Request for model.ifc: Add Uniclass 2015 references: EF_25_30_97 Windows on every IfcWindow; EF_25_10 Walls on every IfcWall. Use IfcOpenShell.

First a look at what the model holds.

```python
import ifcopenshell

model = ifcopenshell.open("model.ifc")
print(model.schema)
print("classifications:", [c.Name for c in model.by_type("IfcClassification")])
for ifc_class in ("IfcDoor", "IfcRoof", "IfcStair", "IfcWall", "IfcWindow"):
    print(ifc_class, len(model.by_type(ifc_class)))
```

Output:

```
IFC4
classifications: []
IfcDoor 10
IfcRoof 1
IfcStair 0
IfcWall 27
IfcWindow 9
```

```python
import ifcopenshell
import ifcopenshell.api.classification

model = ifcopenshell.open("model.ifc")

system = ifcopenshell.api.classification.add_classification(model, classification="Uniclass 2015")

codes = {
    "IfcWindow": ("EF_25_30_97", "Windows"),
    "IfcWall": ("EF_25_10", "Walls"),
}
for ifc_class, (code, name) in codes.items():
    products = model.by_type(ifc_class)
    ifcopenshell.api.classification.add_reference(
        model, products=products, classification=system, identification=code, name=name
    )
    print(code, len(products))

model.write("model-out.ifc")
```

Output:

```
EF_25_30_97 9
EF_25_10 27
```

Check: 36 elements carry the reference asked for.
